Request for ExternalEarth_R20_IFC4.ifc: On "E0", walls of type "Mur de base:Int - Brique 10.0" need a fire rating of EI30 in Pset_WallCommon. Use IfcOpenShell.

First a look at what the model holds.

```python
import ifcopenshell
import ifcopenshell.util.element

model = ifcopenshell.open("ExternalEarth_R20_IFC4.ifc")
print(model.schema)
storey = next(s for s in model.by_type("IfcBuildingStorey") if s.Name == "E0")
walls = [e for e in ifcopenshell.util.element.get_decomposition(storey) if e.is_a("IfcWall")]
seen = {}
for e in walls:
    element_type = ifcopenshell.util.element.get_type(e)
    key = (element_type.Name if element_type != e and element_type else None, ifcopenshell.util.element.get_pset(e, "Pset_WallCommon", "FireRating"))
    seen[key] = seen.get(key, 0) + 1
for (name, value), count in sorted(seen.items(), key=str):
    print(count, "x", name, "|", value)
```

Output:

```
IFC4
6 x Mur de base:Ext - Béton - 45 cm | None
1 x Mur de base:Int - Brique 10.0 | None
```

```python
import ifcopenshell
import ifcopenshell.api.pset
import ifcopenshell.util.element

model = ifcopenshell.open("ExternalEarth_R20_IFC4.ifc")

storey = next(s for s in model.by_type("IfcBuildingStorey") if s.Name == "E0")
walls = [e for e in ifcopenshell.util.element.get_decomposition(storey) if e.is_a("IfcWall")]

count = 0
for e in walls:
    element_type = ifcopenshell.util.element.get_type(e)
    if element_type in (None, e) or element_type.Name != "Mur de base:Int - Brique 10.0":
        continue
    # add_pset returns the element's existing set when there is one.
    pset = ifcopenshell.api.pset.add_pset(model, product=e, name="Pset_WallCommon")
    ifcopenshell.api.pset.edit_pset(model, pset=pset, properties={"FireRating": "EI30"})
    count += 1

print(count, "walls updated")

model.write("ExternalEarth_R20_IFC4_updated.ifc")
```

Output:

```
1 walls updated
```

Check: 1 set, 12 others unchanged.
